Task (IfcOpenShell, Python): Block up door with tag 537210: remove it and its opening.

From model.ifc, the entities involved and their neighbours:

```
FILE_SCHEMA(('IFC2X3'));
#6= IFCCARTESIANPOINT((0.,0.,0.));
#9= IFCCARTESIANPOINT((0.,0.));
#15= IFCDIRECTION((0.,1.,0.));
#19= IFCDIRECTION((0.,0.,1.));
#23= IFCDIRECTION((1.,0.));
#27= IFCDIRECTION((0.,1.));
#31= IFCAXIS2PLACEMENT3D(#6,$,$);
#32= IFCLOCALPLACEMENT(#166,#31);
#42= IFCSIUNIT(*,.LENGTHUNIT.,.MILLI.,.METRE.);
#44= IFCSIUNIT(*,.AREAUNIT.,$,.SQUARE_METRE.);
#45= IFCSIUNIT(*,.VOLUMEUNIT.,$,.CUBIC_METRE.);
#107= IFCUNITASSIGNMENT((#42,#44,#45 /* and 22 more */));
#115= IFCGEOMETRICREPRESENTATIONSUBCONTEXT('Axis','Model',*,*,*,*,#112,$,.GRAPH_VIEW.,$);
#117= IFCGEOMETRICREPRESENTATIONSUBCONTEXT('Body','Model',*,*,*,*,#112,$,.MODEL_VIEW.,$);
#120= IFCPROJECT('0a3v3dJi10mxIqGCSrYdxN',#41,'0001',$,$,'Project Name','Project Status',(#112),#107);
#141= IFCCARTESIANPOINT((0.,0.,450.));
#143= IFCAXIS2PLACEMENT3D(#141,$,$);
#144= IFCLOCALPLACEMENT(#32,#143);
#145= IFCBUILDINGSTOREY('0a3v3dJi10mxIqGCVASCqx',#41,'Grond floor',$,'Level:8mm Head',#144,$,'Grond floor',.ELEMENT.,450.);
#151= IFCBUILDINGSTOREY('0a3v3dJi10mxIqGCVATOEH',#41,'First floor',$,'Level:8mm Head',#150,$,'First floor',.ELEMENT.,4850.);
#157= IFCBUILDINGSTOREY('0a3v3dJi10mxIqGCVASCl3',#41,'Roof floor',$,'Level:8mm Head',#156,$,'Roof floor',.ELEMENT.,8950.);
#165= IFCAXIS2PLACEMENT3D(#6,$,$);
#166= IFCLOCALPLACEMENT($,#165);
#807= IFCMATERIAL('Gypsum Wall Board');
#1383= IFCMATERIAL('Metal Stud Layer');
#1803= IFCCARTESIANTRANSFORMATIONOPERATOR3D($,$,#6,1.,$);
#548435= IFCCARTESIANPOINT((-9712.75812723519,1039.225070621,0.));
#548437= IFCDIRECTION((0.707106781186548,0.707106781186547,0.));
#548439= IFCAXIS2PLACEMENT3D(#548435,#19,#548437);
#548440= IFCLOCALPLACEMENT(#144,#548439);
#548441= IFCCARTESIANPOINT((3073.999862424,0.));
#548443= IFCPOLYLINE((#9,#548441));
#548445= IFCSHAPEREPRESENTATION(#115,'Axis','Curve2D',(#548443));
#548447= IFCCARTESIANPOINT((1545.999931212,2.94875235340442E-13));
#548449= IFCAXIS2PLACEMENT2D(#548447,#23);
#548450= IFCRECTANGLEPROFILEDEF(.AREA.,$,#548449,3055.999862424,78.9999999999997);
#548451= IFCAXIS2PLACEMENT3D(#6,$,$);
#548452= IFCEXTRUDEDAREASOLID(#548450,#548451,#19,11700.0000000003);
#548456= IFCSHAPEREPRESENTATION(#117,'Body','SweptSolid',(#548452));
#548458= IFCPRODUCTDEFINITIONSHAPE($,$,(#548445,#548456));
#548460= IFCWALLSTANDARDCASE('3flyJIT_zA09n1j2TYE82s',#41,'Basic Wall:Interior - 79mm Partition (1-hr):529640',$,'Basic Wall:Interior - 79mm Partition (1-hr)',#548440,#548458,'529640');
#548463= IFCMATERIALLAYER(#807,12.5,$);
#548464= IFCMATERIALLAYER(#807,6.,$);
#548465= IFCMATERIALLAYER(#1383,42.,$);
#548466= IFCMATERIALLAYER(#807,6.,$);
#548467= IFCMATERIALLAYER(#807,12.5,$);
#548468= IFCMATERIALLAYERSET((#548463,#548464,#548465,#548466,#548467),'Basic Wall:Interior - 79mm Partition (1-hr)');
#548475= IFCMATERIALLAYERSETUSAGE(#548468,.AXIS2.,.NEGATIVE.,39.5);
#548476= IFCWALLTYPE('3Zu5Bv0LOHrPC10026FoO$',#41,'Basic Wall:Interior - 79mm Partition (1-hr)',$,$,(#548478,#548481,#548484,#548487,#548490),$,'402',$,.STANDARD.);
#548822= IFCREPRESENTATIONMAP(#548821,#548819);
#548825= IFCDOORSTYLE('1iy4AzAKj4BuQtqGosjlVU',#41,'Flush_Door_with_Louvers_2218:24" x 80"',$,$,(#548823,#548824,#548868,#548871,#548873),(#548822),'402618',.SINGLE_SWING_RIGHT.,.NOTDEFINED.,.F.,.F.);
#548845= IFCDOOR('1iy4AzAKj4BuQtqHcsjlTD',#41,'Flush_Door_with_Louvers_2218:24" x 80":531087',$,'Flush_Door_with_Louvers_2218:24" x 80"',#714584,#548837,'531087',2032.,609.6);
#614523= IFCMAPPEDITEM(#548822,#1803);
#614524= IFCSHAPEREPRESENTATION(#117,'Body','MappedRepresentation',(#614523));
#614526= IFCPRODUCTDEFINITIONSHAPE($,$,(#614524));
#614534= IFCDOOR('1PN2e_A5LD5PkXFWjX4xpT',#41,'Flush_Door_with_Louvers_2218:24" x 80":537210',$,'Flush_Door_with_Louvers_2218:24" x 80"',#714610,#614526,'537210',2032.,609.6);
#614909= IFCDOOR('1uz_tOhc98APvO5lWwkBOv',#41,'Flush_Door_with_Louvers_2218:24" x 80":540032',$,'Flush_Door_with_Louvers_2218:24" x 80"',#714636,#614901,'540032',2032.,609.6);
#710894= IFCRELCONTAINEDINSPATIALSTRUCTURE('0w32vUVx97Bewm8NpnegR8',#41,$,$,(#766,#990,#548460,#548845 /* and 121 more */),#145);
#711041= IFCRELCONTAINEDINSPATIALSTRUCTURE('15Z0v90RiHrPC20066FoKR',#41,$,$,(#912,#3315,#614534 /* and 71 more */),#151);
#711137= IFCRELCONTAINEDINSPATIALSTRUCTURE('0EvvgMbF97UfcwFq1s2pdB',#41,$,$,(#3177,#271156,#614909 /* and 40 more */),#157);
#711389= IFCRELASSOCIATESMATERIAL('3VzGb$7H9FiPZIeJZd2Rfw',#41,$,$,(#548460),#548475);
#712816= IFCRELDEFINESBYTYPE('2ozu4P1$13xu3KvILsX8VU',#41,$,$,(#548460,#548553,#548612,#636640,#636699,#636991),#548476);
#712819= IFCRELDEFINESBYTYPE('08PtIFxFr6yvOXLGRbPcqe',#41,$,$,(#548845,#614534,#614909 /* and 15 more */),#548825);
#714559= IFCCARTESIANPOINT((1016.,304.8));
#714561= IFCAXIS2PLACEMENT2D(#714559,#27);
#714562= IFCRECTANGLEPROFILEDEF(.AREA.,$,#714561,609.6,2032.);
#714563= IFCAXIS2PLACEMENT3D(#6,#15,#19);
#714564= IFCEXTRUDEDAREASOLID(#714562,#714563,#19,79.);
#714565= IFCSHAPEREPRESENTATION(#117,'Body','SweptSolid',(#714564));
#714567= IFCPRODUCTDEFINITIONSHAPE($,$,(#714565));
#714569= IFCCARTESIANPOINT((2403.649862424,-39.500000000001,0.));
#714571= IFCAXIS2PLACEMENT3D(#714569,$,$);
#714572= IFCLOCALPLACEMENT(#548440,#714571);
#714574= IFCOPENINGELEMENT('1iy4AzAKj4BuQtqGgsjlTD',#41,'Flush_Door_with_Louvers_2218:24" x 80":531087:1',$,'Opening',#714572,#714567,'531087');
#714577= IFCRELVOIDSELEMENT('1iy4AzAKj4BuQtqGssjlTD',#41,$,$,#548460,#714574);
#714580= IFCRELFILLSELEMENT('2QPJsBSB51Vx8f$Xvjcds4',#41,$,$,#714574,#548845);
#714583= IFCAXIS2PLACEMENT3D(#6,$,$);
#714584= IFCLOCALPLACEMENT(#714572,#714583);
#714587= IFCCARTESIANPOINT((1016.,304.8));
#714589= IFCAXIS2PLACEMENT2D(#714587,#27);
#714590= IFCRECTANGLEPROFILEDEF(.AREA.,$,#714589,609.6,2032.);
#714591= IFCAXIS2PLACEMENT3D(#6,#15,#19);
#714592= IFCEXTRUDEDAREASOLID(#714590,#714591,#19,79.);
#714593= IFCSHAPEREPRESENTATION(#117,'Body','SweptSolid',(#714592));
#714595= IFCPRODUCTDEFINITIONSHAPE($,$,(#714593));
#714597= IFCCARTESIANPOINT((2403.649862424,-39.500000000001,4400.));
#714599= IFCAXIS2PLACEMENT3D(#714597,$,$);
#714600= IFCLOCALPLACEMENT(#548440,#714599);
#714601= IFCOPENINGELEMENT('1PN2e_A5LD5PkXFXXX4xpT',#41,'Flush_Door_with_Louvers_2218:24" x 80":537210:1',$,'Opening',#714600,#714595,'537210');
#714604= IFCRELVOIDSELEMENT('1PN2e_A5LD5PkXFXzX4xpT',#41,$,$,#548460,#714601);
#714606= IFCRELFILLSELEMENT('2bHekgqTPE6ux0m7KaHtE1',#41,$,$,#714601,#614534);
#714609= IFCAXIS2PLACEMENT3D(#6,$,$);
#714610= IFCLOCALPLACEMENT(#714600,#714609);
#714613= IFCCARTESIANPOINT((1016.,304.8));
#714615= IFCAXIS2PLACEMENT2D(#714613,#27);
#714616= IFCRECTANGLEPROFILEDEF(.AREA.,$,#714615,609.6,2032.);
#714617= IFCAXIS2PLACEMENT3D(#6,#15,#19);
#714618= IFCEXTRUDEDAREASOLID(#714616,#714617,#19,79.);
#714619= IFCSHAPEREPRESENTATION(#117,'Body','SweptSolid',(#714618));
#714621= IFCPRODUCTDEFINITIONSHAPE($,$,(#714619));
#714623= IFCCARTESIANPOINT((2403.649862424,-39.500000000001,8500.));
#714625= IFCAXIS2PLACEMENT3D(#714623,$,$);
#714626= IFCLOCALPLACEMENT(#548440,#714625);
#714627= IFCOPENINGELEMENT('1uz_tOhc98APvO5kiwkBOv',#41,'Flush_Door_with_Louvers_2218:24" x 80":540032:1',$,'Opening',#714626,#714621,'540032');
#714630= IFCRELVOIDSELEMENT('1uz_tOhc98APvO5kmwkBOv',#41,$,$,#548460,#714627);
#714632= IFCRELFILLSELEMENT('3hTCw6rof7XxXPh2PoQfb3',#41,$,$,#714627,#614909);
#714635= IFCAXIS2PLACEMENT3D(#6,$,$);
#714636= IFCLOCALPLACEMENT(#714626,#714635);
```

```python
import ifcopenshell
import ifcopenshell.api.feature
import ifcopenshell.api.root
import ifcopenshell.geom
import ifcopenshell.util.shape

model = ifcopenshell.open("model.ifc")
settings = ifcopenshell.geom.settings()


def volume(element):
    """Net volume in cubic metres, openings subtracted."""
    shape = ifcopenshell.geom.create_shape(settings, element)
    return ifcopenshell.util.shape.get_volume(shape.geometry)


door = model.by_guid("1PN2e_A5LD5PkXFWjX4xpT")
opening = door.FillsVoids[0].RelatingOpeningElement
wall = opening.VoidsElements[0].RelatingBuildingElement
before = volume(wall)

ifcopenshell.api.root.remove_product(model, product=door)
ifcopenshell.api.feature.remove_feature(model, feature=opening)

after = volume(wall)

print(f"wall volume {before:.3f} -> {after:.3f} m3")

model.write("model_rev.ifc")
```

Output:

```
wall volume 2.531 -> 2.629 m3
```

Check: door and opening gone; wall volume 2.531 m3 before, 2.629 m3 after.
